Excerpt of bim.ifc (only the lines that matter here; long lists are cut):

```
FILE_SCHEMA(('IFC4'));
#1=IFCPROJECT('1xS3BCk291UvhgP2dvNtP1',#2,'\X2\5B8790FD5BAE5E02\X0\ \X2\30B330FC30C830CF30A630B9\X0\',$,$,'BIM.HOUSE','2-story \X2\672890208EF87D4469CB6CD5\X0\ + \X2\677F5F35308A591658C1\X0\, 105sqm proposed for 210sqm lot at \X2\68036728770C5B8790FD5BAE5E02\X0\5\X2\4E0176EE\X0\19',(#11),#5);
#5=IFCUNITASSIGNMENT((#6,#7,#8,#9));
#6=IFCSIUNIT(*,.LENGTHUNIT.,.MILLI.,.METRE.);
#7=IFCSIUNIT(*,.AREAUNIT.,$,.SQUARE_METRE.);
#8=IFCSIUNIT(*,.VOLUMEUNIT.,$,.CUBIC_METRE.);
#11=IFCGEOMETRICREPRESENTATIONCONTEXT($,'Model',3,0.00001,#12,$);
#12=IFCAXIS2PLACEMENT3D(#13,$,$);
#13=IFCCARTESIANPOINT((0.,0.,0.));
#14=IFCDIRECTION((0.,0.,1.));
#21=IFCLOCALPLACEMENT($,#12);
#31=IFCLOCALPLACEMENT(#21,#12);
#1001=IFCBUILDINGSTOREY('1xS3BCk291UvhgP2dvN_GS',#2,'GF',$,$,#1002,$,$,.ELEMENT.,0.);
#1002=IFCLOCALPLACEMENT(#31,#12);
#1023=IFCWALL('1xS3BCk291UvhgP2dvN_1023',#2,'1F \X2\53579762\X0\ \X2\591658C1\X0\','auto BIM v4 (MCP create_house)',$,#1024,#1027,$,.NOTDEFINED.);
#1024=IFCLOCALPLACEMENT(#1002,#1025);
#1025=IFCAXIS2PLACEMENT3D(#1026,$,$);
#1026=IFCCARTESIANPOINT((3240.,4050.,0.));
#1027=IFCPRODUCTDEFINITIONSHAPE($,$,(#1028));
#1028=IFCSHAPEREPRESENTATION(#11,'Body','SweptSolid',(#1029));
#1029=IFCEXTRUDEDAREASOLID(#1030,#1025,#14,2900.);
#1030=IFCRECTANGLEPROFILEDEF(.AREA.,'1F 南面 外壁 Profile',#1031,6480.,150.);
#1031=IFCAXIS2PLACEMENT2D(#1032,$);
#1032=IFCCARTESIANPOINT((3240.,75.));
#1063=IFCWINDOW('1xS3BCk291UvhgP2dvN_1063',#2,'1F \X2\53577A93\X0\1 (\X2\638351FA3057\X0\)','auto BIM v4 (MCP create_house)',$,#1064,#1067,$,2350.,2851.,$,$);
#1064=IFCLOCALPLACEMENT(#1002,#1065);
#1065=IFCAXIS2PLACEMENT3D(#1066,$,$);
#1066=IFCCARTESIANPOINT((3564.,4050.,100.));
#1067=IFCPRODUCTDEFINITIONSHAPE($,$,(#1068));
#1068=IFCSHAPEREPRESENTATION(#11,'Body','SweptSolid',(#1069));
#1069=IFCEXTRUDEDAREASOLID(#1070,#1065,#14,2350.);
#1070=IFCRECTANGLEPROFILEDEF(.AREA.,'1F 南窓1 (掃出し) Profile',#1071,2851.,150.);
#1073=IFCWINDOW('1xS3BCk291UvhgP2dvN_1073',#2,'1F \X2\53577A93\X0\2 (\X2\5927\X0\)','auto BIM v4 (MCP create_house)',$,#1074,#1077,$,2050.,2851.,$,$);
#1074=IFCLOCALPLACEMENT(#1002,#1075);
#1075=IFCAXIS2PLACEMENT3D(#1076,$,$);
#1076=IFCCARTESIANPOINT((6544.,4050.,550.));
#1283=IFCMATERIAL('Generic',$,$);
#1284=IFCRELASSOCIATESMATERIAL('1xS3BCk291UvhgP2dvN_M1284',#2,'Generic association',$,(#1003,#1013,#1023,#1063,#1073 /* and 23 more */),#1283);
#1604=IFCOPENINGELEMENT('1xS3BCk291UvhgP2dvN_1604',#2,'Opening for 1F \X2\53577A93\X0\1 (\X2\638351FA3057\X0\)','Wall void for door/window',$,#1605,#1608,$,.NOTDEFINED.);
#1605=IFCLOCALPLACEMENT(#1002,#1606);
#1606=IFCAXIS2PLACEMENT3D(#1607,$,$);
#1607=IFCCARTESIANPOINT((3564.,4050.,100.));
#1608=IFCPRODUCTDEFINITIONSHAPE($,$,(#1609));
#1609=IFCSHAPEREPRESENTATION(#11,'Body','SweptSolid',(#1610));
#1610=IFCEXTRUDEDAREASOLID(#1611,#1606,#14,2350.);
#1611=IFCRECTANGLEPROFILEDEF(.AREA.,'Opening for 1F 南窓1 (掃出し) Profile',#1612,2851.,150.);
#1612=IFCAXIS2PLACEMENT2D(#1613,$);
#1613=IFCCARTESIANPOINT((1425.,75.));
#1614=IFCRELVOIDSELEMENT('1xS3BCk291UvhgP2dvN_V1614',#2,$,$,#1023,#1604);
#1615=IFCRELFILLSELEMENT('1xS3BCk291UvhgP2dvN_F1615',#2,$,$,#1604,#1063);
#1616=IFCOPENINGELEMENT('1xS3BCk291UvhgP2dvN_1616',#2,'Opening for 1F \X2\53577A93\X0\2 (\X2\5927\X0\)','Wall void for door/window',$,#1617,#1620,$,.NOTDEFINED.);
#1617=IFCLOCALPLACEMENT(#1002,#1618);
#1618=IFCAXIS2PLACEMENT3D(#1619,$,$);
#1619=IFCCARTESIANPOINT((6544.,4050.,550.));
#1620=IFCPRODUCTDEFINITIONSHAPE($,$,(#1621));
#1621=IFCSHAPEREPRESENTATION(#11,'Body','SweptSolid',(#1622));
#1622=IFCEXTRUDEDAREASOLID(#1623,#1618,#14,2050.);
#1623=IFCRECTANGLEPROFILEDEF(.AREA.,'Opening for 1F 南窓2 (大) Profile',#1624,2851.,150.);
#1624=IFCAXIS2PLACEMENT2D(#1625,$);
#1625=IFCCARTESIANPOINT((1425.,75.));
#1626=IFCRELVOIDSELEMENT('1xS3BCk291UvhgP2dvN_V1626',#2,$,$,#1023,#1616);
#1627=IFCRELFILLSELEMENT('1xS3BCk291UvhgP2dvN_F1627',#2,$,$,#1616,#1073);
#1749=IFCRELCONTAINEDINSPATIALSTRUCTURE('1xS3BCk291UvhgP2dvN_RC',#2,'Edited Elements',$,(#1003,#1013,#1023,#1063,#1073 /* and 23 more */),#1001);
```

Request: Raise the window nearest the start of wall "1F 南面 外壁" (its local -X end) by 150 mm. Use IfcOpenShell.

```python
import numpy as np
import ifcopenshell
import ifcopenshell.api.geometry
import ifcopenshell.util.placement
import ifcopenshell.util.unit

model = ifcopenshell.open("bim.ifc")
unit_scale = ifcopenshell.util.unit.calculate_unit_scale(model)

window = model.by_guid("1xS3BCk291UvhgP2dvN_1063")
opening = window.FillsVoids[0].RelatingOpeningElement
dz = 150.0

shift = np.array([0.0, 0.0, dz])
# The window is not placed relative to its opening, so move both.
for product in (opening, window):
    matrix = ifcopenshell.util.placement.get_local_placement(product.ObjectPlacement)
    matrix[:3, 3] += shift
    ifcopenshell.api.geometry.edit_object_placement(model, product=product, matrix=matrix, is_si=False)

print(f"moved by {dz * unit_scale:+.3f} m")

model.write("bim_edited.ifc")
```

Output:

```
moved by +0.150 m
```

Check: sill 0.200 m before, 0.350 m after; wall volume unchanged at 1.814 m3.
